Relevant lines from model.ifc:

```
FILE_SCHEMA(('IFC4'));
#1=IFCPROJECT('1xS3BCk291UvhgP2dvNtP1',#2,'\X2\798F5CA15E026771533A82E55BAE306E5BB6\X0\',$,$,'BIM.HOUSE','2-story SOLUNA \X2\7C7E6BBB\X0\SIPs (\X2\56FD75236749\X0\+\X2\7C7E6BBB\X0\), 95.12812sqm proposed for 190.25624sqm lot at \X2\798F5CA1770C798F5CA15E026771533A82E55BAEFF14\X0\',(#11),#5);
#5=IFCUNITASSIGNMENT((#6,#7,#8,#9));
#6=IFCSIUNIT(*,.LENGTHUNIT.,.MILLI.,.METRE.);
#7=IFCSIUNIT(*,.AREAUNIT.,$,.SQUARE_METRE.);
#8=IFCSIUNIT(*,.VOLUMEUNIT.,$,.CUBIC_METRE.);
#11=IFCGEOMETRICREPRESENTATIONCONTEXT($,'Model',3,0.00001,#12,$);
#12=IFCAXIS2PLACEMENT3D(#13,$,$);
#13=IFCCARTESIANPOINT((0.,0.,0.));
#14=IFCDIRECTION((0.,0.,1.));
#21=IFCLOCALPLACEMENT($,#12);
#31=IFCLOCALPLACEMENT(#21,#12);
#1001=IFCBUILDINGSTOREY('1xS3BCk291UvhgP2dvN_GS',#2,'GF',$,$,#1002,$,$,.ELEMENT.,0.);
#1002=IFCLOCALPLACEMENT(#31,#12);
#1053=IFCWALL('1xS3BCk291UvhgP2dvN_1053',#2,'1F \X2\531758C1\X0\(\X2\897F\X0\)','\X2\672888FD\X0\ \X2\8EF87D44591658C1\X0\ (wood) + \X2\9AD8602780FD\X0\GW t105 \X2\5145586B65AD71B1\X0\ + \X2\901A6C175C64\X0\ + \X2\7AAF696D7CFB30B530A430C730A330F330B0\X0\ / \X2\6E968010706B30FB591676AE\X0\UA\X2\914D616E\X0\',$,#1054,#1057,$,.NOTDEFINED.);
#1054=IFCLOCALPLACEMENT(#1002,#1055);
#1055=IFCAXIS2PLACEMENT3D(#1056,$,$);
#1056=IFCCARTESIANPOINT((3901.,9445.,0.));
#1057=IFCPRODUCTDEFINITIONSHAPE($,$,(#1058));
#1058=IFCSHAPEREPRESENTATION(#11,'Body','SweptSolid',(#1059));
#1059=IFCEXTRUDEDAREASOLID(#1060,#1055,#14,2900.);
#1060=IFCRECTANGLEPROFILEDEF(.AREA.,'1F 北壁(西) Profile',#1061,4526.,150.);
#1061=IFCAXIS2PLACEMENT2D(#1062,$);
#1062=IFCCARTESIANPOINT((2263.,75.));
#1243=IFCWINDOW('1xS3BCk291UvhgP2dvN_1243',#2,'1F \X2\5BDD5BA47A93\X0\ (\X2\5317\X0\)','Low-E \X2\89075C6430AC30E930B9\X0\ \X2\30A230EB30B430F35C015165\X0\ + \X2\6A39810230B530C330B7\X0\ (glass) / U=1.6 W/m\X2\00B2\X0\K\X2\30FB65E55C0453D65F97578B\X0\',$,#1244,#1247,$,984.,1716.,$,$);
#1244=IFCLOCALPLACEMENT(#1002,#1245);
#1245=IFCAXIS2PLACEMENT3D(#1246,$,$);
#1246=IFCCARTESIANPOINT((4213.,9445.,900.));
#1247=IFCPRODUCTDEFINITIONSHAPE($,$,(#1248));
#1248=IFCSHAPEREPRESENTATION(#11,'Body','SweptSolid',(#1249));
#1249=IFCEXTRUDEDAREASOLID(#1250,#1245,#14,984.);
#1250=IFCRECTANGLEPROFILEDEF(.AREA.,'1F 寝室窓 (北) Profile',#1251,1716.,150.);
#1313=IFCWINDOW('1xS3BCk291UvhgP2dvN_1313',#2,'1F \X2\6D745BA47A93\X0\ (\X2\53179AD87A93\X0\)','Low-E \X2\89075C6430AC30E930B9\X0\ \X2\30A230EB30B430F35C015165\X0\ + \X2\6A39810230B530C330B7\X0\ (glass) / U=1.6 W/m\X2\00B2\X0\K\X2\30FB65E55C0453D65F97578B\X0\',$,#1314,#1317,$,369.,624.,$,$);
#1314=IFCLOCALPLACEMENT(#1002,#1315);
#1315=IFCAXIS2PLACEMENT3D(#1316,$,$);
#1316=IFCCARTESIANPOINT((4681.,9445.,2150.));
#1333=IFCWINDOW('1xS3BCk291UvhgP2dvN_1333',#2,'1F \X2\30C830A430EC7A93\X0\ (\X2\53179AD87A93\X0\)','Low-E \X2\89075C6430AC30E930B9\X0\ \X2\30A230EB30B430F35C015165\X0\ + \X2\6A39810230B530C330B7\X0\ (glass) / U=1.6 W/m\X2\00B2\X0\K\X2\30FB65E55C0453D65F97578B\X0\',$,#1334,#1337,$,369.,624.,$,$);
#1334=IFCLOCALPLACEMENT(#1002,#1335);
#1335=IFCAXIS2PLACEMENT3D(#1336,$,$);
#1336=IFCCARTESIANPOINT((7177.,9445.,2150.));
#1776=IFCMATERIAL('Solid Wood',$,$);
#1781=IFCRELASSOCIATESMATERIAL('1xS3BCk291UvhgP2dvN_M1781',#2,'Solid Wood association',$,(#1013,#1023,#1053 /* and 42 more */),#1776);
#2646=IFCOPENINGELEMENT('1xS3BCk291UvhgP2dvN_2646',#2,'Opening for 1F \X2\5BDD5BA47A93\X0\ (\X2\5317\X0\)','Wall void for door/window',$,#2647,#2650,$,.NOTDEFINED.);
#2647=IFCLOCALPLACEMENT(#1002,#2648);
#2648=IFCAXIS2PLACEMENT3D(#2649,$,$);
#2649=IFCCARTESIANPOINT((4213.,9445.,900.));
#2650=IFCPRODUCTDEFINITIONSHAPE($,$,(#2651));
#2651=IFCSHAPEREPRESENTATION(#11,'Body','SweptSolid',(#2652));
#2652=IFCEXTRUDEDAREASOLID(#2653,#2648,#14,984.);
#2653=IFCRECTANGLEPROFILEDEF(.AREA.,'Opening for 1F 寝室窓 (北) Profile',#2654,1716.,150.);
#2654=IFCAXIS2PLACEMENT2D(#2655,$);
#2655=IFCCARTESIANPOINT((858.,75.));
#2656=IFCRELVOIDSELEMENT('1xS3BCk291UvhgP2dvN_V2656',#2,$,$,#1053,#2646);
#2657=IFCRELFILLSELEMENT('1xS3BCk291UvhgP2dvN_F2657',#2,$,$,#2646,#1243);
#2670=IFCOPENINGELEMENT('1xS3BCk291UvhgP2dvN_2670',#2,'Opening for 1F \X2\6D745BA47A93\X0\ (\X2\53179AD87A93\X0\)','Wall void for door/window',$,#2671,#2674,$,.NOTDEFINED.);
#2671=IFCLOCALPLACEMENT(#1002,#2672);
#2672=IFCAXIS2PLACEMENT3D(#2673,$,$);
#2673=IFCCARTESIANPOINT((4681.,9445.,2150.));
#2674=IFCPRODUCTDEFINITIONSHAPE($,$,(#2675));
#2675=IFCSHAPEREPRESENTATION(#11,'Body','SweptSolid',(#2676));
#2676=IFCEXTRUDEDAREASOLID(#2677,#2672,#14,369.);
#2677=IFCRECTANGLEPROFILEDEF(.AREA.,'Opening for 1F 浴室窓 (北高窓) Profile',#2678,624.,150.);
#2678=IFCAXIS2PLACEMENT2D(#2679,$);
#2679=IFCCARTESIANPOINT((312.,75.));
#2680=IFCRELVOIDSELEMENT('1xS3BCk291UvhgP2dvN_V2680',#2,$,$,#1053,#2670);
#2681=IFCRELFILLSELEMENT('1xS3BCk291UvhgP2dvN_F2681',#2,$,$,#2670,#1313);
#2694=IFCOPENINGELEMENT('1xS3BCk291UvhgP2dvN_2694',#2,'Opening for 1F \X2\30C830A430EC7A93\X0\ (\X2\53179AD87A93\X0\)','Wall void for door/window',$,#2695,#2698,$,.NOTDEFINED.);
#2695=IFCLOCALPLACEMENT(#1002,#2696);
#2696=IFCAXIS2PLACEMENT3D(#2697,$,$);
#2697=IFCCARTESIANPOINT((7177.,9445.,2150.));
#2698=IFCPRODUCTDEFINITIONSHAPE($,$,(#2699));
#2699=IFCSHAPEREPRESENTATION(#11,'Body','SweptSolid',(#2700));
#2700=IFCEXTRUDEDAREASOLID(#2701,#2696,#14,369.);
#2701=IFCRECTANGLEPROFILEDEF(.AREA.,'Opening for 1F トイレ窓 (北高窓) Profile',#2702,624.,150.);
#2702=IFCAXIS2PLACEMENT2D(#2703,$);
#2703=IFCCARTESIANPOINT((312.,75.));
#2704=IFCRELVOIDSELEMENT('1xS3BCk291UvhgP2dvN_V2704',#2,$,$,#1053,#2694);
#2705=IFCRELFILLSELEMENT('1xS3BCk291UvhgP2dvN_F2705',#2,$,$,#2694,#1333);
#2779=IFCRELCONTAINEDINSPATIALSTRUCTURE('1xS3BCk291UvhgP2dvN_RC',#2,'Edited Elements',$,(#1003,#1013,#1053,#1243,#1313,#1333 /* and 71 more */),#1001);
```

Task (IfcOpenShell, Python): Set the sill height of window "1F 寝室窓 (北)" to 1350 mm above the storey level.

```python
import numpy as np
import ifcopenshell
import ifcopenshell.api.geometry
import ifcopenshell.geom
import ifcopenshell.util.element
import ifcopenshell.util.placement
import ifcopenshell.util.shape
import ifcopenshell.util.unit

model = ifcopenshell.open("model.ifc")
unit_scale = ifcopenshell.util.unit.calculate_unit_scale(model)

window = model.by_id(1243)
opening = window.FillsVoids[0].RelatingOpeningElement
storey = ifcopenshell.util.element.get_container(window, ifc_class="IfcBuildingStorey")
level = ifcopenshell.util.placement.get_local_placement(storey.ObjectPlacement)[2, 3]

# The opening's origin need not be at the sill, so measure its lowest point.
shape = ifcopenshell.geom.create_shape(ifcopenshell.geom.settings(), opening)
bottom = ifcopenshell.util.shape.get_shape_bottom_elevation(shape, shape.geometry) / unit_scale
dz = level + 1.35 / unit_scale - bottom

shift = np.array([0.0, 0.0, dz])
# The window is not placed relative to its opening, so move both.
for product in (opening, window):
    matrix = ifcopenshell.util.placement.get_local_placement(product.ObjectPlacement)
    matrix[:3, 3] += shift
    ifcopenshell.api.geometry.edit_object_placement(model, product=product, matrix=matrix, is_si=False)

print(f"moved by {dz * unit_scale:+.3f} m")

model.write("model_v2.ifc")
```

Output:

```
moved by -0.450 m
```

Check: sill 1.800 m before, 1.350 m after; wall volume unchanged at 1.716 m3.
